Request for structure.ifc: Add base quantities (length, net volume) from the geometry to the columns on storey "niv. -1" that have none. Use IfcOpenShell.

First a look at what the model holds.

```python
import ifcopenshell
import ifcopenshell.util.element
import ifcopenshell.util.unit

model = ifcopenshell.open("structure.ifc")
print(model.schema)
for unit_type in ("LENGTHUNIT", "AREAUNIT", "VOLUMEUNIT"):
    print(unit_type, ifcopenshell.util.unit.calculate_unit_scale(model, unit_type))
storey = next(s for s in model.by_type("IfcBuildingStorey") if s.Name == "niv. -1")
columns = [e for e in ifcopenshell.util.element.get_decomposition(storey) if e.is_a("IfcColumn")]
for e in sorted(columns, key=lambda e: e.id()):
    print(e.id(), e.is_a(), e.Name, list(ifcopenshell.util.element.get_psets(e, qtos_only=True)), sep=" | ")
```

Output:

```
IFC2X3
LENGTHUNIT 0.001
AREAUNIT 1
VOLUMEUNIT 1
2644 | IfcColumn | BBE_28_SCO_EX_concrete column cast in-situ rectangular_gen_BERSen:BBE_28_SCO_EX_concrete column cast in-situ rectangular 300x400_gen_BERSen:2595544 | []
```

```python
import ifcopenshell
import ifcopenshell.api.pset
import ifcopenshell.geom
import ifcopenshell.util.element
import ifcopenshell.util.shape
import ifcopenshell.util.unit

model = ifcopenshell.open("structure.ifc")
unit_scale = ifcopenshell.util.unit.calculate_unit_scale(model)
volume_scale = ifcopenshell.util.unit.calculate_unit_scale(model, "VOLUMEUNIT")
settings = ifcopenshell.geom.settings()

storey = next(s for s in model.by_type("IfcBuildingStorey") if s.Name == "niv. -1")
columns = [e for e in ifcopenshell.util.element.get_decomposition(storey) if e.is_a("IfcColumn")]

for e in sorted(columns, key=lambda e: e.id()):
    if ifcopenshell.util.element.get_psets(e, qtos_only=True, should_inherit=False):
        continue
    # Geometry comes back in metres, in the element's own axes.
    shape = ifcopenshell.geom.create_shape(settings, e)
    values = {
        "Length": ifcopenshell.util.shape.get_z(shape.geometry) / unit_scale,
        "NetVolume": ifcopenshell.util.shape.get_volume(shape.geometry) / volume_scale,
    }
    qto = ifcopenshell.api.pset.add_qto(model, product=e, name="BaseQuantities")
    ifcopenshell.api.pset.edit_qto(model, qto=qto, properties=values)
    print(e.id(), {k: round(v, 3) for k, v in values.items()})

model.write("structure_edited.ifc")
```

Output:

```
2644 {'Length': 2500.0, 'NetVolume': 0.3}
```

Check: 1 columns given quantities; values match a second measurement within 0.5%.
